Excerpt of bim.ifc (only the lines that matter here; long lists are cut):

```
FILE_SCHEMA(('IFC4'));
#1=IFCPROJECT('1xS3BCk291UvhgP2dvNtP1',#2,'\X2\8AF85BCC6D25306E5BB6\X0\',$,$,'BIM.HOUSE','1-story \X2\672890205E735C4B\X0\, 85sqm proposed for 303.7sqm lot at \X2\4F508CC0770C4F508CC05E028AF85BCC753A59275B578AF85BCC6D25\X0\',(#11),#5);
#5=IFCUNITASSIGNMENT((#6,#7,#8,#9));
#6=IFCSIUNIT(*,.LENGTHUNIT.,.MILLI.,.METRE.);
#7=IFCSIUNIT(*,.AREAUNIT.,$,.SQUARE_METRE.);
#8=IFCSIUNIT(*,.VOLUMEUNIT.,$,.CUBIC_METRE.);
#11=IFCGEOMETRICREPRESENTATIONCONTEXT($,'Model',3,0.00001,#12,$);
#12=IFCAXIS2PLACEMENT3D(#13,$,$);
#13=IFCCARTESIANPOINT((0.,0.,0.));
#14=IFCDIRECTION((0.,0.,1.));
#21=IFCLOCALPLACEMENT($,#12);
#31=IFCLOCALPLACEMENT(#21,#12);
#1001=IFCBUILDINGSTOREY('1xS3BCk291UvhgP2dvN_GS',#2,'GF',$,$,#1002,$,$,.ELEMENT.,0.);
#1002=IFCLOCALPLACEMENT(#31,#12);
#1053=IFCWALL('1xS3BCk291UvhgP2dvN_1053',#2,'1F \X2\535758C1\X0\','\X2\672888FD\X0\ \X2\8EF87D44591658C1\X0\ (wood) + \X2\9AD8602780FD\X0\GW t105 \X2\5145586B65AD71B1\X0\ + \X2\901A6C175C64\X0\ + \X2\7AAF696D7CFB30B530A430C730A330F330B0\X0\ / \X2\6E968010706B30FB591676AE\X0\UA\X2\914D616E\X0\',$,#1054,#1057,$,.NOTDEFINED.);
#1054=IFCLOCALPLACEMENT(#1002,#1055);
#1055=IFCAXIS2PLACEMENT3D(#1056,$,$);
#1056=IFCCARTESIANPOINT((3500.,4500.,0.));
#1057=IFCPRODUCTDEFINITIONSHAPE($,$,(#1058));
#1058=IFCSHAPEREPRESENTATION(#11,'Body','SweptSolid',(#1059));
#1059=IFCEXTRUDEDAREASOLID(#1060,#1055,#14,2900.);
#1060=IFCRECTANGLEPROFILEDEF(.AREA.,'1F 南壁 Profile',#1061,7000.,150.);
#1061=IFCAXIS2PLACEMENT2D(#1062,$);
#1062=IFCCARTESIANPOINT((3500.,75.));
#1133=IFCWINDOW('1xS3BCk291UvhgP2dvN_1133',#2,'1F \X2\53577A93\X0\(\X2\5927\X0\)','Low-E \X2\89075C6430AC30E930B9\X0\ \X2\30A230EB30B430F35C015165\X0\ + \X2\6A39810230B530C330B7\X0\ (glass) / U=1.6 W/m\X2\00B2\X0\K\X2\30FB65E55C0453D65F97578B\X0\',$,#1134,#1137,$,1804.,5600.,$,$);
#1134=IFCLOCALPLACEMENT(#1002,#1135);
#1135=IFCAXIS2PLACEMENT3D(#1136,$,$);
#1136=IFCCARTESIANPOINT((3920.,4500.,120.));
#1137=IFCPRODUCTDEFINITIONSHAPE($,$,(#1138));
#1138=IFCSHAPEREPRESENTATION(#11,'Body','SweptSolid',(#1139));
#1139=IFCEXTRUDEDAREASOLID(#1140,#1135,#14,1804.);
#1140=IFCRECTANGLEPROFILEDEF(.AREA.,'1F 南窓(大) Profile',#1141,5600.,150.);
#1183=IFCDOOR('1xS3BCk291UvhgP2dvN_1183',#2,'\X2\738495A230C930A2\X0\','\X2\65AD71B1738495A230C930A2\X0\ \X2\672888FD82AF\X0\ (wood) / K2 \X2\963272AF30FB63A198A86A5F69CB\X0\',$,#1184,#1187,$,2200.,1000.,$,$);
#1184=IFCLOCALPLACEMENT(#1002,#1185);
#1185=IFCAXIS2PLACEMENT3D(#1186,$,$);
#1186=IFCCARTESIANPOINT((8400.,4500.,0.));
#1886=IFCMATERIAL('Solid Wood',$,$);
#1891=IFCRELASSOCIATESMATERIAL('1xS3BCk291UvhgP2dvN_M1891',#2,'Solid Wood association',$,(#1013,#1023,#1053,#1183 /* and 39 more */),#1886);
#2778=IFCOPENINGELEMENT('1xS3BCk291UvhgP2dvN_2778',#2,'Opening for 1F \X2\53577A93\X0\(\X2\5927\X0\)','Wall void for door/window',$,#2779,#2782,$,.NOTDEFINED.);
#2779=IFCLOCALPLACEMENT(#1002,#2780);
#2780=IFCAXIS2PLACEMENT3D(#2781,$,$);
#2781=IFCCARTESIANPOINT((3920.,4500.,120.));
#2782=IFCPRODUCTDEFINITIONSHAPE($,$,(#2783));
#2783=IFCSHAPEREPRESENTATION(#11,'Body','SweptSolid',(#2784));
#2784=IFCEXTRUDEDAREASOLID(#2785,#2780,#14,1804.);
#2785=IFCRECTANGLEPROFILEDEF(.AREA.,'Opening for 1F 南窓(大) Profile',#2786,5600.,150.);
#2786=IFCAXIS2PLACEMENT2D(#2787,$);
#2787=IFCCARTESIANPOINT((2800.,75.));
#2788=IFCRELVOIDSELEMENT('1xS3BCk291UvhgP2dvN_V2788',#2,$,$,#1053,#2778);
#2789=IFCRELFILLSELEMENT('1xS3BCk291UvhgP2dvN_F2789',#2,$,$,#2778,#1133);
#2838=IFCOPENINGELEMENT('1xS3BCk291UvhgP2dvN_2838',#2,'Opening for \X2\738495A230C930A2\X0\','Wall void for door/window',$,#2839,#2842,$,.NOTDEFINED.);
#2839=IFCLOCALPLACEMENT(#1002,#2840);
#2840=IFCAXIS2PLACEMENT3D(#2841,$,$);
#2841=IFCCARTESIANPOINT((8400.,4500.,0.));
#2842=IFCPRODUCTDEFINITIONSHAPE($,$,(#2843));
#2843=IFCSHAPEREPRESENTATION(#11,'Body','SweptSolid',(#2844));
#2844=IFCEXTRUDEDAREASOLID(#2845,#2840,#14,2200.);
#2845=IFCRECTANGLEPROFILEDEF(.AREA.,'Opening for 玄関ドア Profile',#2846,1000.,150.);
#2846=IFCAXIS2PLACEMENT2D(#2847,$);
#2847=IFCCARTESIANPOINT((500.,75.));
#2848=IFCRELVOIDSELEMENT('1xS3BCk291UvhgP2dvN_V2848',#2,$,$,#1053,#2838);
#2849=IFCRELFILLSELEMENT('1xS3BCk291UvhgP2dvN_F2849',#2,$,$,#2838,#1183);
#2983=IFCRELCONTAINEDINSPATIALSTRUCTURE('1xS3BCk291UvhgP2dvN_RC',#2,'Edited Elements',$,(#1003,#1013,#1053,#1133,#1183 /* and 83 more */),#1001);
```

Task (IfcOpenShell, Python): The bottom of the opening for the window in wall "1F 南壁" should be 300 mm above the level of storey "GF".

```python
import numpy as np
import ifcopenshell
import ifcopenshell.api.geometry
import ifcopenshell.geom
import ifcopenshell.util.element
import ifcopenshell.util.placement
import ifcopenshell.util.shape
import ifcopenshell.util.unit

model = ifcopenshell.open("bim.ifc")
unit_scale = ifcopenshell.util.unit.calculate_unit_scale(model)

window = model.by_guid("1xS3BCk291UvhgP2dvN_1133")
opening = window.FillsVoids[0].RelatingOpeningElement
storey = ifcopenshell.util.element.get_container(window, ifc_class="IfcBuildingStorey")
level = ifcopenshell.util.placement.get_local_placement(storey.ObjectPlacement)[2, 3]

# The opening's origin need not be at the sill, so measure its lowest point.
shape = ifcopenshell.geom.create_shape(ifcopenshell.geom.settings(), opening)
bottom = ifcopenshell.util.shape.get_shape_bottom_elevation(shape, shape.geometry) / unit_scale
dz = level + 300.0 - bottom

shift = np.array([0.0, 0.0, dz])
# The window is not placed relative to its opening, so move both.
for product in (opening, window):
    matrix = ifcopenshell.util.placement.get_local_placement(product.ObjectPlacement)
    matrix[:3, 3] += shift
    ifcopenshell.api.geometry.edit_object_placement(model, product=product, matrix=matrix, is_si=False)

print(f"moved by {dz * unit_scale:+.3f} m")

model.write("bim_rev.ifc")
```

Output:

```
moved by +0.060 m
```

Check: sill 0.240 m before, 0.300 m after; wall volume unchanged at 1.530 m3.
